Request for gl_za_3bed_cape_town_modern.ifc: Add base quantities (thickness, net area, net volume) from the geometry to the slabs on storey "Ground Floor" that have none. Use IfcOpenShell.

First a look at what the model holds.

```python
import ifcopenshell
import ifcopenshell.util.element
import ifcopenshell.util.unit

model = ifcopenshell.open("gl_za_3bed_cape_town_modern.ifc")
print(model.schema)
for unit_type in ("LENGTHUNIT", "AREAUNIT", "VOLUMEUNIT"):
    print(unit_type, ifcopenshell.util.unit.calculate_unit_scale(model, unit_type))
storey = next(s for s in model.by_type("IfcBuildingStorey") if s.Name == "Ground Floor")
slabs = [e for e in ifcopenshell.util.element.get_decomposition(storey) if e.is_a("IfcSlab")]
for e in sorted(slabs, key=lambda e: e.id()):
    print(e.id(), e.is_a(), e.Name, list(ifcopenshell.util.element.get_psets(e, qtos_only=True)), sep=" | ")
```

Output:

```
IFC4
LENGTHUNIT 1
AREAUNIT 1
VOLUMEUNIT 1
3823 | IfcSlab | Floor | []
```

```python
import ifcopenshell
import ifcopenshell.api.pset
import ifcopenshell.geom
import ifcopenshell.util.element
import ifcopenshell.util.shape
import ifcopenshell.util.unit

model = ifcopenshell.open("gl_za_3bed_cape_town_modern.ifc")
unit_scale = ifcopenshell.util.unit.calculate_unit_scale(model)
area_scale = ifcopenshell.util.unit.calculate_unit_scale(model, "AREAUNIT")
volume_scale = ifcopenshell.util.unit.calculate_unit_scale(model, "VOLUMEUNIT")
settings = ifcopenshell.geom.settings()

storey = next(s for s in model.by_type("IfcBuildingStorey") if s.Name == "Ground Floor")
slabs = [e for e in ifcopenshell.util.element.get_decomposition(storey) if e.is_a("IfcSlab")]

for e in sorted(slabs, key=lambda e: e.id()):
    if ifcopenshell.util.element.get_psets(e, qtos_only=True, should_inherit=False):
        continue
    # Geometry comes back in metres, in the element's own axes.
    shape = ifcopenshell.geom.create_shape(settings, e)
    values = {
        "Width": ifcopenshell.util.shape.get_z(shape.geometry) / unit_scale,
        "NetArea": ifcopenshell.util.shape.get_footprint_area(shape.geometry) / area_scale,
        "NetVolume": ifcopenshell.util.shape.get_volume(shape.geometry) / volume_scale,
    }
    qto = ifcopenshell.api.pset.add_qto(model, product=e, name="Qto_SlabBaseQuantities")
    ifcopenshell.api.pset.edit_qto(model, qto=qto, properties=values)
    print(e.id(), {k: round(v, 3) for k, v in values.items()})

model.write("gl_za_3bed_cape_town_modern_edited.ifc")
```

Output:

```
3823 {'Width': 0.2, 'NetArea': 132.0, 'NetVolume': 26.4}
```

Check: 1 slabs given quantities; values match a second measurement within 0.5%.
